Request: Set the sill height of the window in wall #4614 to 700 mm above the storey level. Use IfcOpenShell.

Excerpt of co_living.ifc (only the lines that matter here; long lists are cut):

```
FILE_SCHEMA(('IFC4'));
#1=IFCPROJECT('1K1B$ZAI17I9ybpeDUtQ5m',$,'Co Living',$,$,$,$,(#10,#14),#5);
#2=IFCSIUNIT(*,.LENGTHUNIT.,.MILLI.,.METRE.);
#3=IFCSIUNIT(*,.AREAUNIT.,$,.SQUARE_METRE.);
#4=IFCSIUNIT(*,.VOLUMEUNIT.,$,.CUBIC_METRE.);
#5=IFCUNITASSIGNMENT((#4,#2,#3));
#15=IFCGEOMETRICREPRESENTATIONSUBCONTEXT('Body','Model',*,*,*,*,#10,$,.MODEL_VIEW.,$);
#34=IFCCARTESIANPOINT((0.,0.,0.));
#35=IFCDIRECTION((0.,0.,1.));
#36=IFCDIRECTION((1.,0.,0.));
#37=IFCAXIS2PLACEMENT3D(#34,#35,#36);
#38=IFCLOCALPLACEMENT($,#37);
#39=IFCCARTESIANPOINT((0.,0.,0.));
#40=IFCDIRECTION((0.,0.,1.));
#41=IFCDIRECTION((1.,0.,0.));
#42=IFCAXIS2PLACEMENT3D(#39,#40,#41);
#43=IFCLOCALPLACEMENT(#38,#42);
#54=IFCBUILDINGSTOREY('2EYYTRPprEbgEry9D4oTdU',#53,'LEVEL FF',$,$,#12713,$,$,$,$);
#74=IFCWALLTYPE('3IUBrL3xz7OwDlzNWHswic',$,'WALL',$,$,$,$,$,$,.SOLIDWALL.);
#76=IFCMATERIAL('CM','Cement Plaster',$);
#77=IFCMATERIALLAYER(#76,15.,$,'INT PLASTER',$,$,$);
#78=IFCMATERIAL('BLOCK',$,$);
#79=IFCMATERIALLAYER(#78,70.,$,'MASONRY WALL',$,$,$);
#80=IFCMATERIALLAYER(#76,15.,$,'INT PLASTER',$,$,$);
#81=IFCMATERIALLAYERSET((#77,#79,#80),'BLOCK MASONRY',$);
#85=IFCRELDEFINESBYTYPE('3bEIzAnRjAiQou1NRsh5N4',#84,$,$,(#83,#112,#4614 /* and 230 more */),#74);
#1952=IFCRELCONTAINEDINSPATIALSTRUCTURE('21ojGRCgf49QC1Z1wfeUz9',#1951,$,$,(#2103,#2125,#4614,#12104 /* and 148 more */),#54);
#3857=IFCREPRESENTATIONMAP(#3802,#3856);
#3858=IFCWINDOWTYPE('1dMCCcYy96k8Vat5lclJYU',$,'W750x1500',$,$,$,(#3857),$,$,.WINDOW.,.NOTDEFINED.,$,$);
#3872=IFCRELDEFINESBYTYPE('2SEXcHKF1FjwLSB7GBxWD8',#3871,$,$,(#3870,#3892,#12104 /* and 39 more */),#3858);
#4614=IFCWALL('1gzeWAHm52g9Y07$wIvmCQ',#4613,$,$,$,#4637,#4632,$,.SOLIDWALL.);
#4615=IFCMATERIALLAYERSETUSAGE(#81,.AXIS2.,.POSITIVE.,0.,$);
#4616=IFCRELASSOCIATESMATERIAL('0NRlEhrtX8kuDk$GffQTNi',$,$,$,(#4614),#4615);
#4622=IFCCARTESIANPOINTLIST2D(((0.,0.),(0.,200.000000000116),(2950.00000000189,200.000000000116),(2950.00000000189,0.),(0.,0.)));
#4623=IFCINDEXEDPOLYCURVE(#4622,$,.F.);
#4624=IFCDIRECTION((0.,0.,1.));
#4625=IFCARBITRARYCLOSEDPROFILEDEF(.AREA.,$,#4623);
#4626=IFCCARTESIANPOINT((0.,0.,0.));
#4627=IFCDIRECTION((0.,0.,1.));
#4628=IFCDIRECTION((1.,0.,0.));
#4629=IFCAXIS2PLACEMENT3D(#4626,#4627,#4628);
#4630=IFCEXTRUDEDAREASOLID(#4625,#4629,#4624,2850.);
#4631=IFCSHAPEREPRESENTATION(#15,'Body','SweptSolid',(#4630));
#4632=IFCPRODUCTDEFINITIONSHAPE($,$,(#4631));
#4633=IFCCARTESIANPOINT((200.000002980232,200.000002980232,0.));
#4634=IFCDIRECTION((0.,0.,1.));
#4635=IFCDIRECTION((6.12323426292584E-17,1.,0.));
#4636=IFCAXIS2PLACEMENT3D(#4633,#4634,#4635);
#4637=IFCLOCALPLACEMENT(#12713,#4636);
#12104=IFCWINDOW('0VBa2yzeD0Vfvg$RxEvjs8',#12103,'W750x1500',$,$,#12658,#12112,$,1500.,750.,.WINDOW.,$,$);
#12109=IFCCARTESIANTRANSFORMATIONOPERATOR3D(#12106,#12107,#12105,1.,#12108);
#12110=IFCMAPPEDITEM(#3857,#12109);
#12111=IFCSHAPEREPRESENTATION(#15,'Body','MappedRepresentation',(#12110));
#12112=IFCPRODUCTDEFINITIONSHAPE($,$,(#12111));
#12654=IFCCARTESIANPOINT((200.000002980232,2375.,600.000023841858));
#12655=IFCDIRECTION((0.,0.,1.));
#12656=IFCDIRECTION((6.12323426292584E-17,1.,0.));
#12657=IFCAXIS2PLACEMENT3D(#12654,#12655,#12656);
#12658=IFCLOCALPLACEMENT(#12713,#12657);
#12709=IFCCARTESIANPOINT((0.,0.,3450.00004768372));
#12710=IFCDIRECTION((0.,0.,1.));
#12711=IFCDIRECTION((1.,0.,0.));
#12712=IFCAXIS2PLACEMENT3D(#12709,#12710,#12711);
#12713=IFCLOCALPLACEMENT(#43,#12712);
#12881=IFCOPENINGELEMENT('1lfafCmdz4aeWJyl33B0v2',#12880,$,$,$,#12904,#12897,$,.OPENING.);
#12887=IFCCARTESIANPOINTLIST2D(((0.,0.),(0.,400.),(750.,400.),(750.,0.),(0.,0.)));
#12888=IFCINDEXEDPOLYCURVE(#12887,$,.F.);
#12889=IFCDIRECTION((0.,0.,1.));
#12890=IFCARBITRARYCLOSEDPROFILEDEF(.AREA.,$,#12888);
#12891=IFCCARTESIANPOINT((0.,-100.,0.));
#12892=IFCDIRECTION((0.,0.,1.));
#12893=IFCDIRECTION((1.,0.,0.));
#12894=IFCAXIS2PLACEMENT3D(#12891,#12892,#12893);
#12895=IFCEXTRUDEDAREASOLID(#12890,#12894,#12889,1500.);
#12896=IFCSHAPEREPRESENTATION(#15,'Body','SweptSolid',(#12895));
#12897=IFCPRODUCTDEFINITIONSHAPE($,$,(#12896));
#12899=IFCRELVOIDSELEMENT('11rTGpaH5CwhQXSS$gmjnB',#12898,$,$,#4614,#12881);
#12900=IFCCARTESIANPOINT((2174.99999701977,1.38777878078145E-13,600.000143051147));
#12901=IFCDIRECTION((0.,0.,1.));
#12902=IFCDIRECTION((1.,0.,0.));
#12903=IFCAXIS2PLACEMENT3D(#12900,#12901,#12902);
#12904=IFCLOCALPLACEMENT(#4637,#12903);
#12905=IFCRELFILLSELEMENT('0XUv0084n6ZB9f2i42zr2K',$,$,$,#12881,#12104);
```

```python
import numpy as np
import ifcopenshell
import ifcopenshell.api.geometry
import ifcopenshell.geom
import ifcopenshell.util.element
import ifcopenshell.util.placement
import ifcopenshell.util.shape
import ifcopenshell.util.unit

model = ifcopenshell.open("co_living.ifc")
unit_scale = ifcopenshell.util.unit.calculate_unit_scale(model)

window = model.by_guid("0VBa2yzeD0Vfvg$RxEvjs8")
opening = window.FillsVoids[0].RelatingOpeningElement
storey = ifcopenshell.util.element.get_container(window, ifc_class="IfcBuildingStorey")
level = ifcopenshell.util.placement.get_local_placement(storey.ObjectPlacement)[2, 3]

# The opening's origin need not be at the sill, so measure its lowest point.
shape = ifcopenshell.geom.create_shape(ifcopenshell.geom.settings(), opening)
bottom = ifcopenshell.util.shape.get_shape_bottom_elevation(shape, shape.geometry) / unit_scale
dz = level + 700.0 - bottom

shift = np.array([0.0, 0.0, dz])
# The window is not placed relative to its opening, so move both.
for product in (opening, window):
    matrix = ifcopenshell.util.placement.get_local_placement(product.ObjectPlacement)
    matrix[:3, 3] += shift
    ifcopenshell.api.geometry.edit_object_placement(model, product=product, matrix=matrix, is_si=False)

print(f"moved by {dz * unit_scale:+.3f} m")

model.write("co_living_rev.ifc")
```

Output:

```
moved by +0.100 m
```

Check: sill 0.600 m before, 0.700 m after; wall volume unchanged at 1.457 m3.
